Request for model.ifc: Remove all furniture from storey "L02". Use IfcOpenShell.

First a look at what the model holds.

```python
import ifcopenshell
import ifcopenshell.util.element

model = ifcopenshell.open("model.ifc")
print(model.schema)
storey = next(s for s in model.by_type("IfcBuildingStorey") if s.Name == "L02")
furniture = [e for e in ifcopenshell.util.element.get_decomposition(storey) if e.is_a("IfcFurnishingElement")]
seen = {}
for e in furniture:
    element_type = ifcopenshell.util.element.get_type(e)
    name = element_type.Name if element_type not in (None, e) else None
    seen[name] = seen.get(name, 0) + 1
for name, count in sorted(seen.items(), key=str):
    print(count, "x", name)
```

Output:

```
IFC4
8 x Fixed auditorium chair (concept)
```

```python
import ifcopenshell
import ifcopenshell.api.root
import ifcopenshell.util.element

model = ifcopenshell.open("model.ifc")

storey = next(s for s in model.by_type("IfcBuildingStorey") if s.Name == "L02")
furniture = [e for e in ifcopenshell.util.element.get_decomposition(storey) if e.is_a("IfcFurnishingElement")]

for e in furniture:
    ifcopenshell.api.root.remove_product(model, product=e)
print(len(furniture), "removed")

model.write("model_v2.ifc")
```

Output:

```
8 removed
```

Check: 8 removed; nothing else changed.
